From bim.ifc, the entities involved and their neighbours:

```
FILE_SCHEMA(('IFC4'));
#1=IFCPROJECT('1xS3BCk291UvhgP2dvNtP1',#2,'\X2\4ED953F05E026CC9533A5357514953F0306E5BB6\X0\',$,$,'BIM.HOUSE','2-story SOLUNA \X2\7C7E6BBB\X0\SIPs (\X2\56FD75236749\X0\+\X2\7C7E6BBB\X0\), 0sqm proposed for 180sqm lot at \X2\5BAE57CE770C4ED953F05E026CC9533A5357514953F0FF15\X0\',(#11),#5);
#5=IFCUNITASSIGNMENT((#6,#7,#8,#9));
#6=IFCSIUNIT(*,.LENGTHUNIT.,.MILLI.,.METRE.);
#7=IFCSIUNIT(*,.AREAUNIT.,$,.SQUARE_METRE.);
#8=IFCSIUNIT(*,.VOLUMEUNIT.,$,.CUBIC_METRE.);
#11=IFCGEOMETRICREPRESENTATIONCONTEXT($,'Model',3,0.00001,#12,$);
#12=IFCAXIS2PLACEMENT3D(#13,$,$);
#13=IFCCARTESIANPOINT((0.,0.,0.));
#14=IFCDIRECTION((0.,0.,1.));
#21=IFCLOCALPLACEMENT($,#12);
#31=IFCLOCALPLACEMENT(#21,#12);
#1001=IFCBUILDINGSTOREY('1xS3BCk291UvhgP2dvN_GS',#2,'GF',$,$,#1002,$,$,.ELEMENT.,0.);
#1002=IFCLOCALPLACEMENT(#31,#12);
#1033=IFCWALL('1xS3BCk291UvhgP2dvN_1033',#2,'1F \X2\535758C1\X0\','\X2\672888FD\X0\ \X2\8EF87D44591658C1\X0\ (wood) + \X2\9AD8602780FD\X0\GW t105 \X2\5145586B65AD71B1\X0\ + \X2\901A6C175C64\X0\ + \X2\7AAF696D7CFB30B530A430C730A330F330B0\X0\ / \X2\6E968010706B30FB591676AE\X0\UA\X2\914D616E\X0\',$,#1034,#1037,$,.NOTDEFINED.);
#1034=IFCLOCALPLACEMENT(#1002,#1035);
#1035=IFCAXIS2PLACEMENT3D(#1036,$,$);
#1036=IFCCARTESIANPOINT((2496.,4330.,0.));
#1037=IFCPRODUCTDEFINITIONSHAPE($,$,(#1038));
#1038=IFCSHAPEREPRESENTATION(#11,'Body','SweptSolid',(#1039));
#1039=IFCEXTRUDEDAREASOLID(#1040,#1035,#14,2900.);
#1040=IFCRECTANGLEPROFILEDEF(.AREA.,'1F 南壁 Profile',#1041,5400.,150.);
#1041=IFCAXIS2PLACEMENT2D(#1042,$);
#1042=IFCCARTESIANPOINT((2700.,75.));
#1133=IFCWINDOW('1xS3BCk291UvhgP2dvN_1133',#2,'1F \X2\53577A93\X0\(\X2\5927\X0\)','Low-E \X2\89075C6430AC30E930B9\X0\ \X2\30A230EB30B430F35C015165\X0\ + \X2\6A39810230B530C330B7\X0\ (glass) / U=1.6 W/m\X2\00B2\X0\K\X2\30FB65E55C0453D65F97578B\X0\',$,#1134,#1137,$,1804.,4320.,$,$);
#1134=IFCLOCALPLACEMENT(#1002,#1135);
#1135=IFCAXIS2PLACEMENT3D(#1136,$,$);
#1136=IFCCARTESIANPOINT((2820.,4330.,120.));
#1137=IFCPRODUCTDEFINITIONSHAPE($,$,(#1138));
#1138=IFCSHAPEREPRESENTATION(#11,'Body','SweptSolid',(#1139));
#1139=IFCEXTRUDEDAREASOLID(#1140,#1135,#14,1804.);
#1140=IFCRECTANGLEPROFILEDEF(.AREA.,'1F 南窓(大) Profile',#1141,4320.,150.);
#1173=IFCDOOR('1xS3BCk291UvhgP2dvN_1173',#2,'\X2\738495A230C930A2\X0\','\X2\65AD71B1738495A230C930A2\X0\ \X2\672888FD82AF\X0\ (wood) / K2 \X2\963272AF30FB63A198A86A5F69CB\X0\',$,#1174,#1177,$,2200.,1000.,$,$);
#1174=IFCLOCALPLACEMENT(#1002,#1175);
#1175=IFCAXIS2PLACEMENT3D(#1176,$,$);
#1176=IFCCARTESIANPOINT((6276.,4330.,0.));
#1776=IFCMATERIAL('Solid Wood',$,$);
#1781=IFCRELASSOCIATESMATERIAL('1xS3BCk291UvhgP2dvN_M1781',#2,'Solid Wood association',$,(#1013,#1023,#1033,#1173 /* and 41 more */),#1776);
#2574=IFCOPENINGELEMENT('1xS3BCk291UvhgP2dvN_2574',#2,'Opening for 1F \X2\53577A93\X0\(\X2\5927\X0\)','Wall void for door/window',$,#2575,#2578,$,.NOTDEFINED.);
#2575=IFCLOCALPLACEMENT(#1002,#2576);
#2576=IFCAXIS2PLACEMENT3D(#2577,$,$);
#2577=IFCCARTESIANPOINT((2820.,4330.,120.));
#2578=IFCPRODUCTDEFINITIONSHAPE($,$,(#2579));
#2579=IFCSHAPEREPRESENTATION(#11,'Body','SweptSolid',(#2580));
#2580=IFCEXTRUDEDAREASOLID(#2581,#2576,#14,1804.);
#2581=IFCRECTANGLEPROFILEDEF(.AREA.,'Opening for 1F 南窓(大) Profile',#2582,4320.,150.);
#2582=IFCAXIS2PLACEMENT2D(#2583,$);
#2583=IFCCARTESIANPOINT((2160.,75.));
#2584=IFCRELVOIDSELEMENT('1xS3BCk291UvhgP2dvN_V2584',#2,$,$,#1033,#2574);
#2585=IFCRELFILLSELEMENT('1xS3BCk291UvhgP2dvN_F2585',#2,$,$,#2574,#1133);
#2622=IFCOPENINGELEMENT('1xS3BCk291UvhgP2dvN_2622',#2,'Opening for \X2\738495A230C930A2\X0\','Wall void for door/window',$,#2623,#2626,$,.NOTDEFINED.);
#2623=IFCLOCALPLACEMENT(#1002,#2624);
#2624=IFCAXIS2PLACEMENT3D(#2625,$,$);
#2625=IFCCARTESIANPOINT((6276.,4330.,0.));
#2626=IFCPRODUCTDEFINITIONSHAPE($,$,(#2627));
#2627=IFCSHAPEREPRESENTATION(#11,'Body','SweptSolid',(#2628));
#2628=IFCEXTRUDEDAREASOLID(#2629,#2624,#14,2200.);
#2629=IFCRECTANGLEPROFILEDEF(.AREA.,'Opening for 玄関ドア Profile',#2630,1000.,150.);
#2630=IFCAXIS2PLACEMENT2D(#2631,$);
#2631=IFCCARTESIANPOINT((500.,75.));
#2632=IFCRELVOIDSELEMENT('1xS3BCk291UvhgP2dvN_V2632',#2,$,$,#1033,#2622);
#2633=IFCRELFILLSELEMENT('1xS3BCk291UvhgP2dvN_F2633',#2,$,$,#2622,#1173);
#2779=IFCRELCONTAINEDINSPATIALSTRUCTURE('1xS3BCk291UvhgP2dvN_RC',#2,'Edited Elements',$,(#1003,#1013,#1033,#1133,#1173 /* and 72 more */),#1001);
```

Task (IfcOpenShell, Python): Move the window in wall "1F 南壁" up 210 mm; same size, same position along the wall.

```python
import numpy as np
import ifcopenshell
import ifcopenshell.api.geometry
import ifcopenshell.util.placement
import ifcopenshell.util.unit

model = ifcopenshell.open("bim.ifc")
unit_scale = ifcopenshell.util.unit.calculate_unit_scale(model)

window = model.by_id(1133)
opening = window.FillsVoids[0].RelatingOpeningElement
dz = 210.0

shift = np.array([0.0, 0.0, dz])
# The window is not placed relative to its opening, so move both.
for product in (opening, window):
    matrix = ifcopenshell.util.placement.get_local_placement(product.ObjectPlacement)
    matrix[:3, 3] += shift
    ifcopenshell.api.geometry.edit_object_placement(model, product=product, matrix=matrix, is_si=False)

print(f"moved by {dz * unit_scale:+.3f} m")

model.write("bim-out.ifc")
```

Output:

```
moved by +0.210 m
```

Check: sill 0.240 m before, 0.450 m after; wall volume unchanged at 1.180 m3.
